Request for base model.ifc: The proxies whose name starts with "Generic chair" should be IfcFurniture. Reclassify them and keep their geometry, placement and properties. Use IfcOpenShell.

First a look at what the model holds.

```python
import re

import ifcopenshell

model = ifcopenshell.open("base model.ifc")
print(model.schema)
seen = {}
for e in model.by_type("IfcBuildingElementProxy"):
    name = re.sub(r":\d+(:\d+)?$", "", e.Name or "")  # drop the element id that some exporters append
    seen[name] = seen.get(name, 0) + 1
for name, count in sorted(seen.items()):
    print(count, "x", name)
```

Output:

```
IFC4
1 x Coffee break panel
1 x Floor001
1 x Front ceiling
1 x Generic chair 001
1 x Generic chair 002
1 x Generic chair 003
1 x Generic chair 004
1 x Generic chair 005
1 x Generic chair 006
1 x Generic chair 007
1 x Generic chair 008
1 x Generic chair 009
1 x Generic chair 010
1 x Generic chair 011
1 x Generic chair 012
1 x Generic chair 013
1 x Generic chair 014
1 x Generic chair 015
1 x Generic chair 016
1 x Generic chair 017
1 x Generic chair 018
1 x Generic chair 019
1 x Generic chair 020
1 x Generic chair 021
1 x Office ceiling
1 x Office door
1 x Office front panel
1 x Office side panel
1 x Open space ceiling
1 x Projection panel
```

```python
import ifcopenshell
import ifcopenshell.api.root

model = ifcopenshell.open("base model.ifc")

proxies = [e.id() for e in model.by_type("IfcBuildingElementProxy") if (e.Name or "").startswith("Generic chair")]
for step_id in proxies:
    proxy = model.by_id(step_id)
    ifcopenshell.api.root.reassign_class(model, product=proxy, ifc_class="IfcFurniture")

print(sum(model.by_id(i).is_a("IfcFurniture") for i in proxies), "reclassified")

model.write("base model_updated.ifc")
```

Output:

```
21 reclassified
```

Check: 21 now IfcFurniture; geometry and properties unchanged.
